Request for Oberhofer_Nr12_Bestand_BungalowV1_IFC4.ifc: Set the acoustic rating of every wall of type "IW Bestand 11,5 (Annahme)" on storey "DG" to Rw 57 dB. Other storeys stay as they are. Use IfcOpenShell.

First a look at what the model holds.

```python
import ifcopenshell
import ifcopenshell.util.element

model = ifcopenshell.open("Oberhofer_Nr12_Bestand_BungalowV1_IFC4.ifc")
print(model.schema)
storey = next(s for s in model.by_type("IfcBuildingStorey") if s.Name == "DG")
walls = [e for e in ifcopenshell.util.element.get_decomposition(storey) if e.is_a("IfcWall")]
seen = {}
for e in walls:
    element_type = ifcopenshell.util.element.get_type(e)
    key = (element_type.Name if element_type != e and element_type else None, ifcopenshell.util.element.get_pset(e, "Pset_WallCommon", "AcousticRating"))
    seen[key] = seen.get(key, 0) + 1
for (name, value), count in sorted(seen.items(), key=str):
    print(count, "x", name, "|", value)
```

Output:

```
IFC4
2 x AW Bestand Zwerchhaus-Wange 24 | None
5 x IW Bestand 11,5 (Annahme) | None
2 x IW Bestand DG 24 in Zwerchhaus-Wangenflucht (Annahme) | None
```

```python
import ifcopenshell
import ifcopenshell.api.pset
import ifcopenshell.util.element

model = ifcopenshell.open("Oberhofer_Nr12_Bestand_BungalowV1_IFC4.ifc")

storey = next(s for s in model.by_type("IfcBuildingStorey") if s.Name == "DG")
walls = [e for e in ifcopenshell.util.element.get_decomposition(storey) if e.is_a("IfcWall")]

count = 0
for e in walls:
    element_type = ifcopenshell.util.element.get_type(e)
    if element_type in (None, e) or element_type.Name != "IW Bestand 11,5 (Annahme)":
        continue
    # add_pset returns the element's existing set when there is one.
    pset = ifcopenshell.api.pset.add_pset(model, product=e, name="Pset_WallCommon")
    ifcopenshell.api.pset.edit_pset(model, pset=pset, properties={"AcousticRating": "Rw 57 dB"})
    count += 1

print(count, "walls updated")

model.write("Oberhofer_Nr12_Bestand_BungalowV1_IFC4-out.ifc")
```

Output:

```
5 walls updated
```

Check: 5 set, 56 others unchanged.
